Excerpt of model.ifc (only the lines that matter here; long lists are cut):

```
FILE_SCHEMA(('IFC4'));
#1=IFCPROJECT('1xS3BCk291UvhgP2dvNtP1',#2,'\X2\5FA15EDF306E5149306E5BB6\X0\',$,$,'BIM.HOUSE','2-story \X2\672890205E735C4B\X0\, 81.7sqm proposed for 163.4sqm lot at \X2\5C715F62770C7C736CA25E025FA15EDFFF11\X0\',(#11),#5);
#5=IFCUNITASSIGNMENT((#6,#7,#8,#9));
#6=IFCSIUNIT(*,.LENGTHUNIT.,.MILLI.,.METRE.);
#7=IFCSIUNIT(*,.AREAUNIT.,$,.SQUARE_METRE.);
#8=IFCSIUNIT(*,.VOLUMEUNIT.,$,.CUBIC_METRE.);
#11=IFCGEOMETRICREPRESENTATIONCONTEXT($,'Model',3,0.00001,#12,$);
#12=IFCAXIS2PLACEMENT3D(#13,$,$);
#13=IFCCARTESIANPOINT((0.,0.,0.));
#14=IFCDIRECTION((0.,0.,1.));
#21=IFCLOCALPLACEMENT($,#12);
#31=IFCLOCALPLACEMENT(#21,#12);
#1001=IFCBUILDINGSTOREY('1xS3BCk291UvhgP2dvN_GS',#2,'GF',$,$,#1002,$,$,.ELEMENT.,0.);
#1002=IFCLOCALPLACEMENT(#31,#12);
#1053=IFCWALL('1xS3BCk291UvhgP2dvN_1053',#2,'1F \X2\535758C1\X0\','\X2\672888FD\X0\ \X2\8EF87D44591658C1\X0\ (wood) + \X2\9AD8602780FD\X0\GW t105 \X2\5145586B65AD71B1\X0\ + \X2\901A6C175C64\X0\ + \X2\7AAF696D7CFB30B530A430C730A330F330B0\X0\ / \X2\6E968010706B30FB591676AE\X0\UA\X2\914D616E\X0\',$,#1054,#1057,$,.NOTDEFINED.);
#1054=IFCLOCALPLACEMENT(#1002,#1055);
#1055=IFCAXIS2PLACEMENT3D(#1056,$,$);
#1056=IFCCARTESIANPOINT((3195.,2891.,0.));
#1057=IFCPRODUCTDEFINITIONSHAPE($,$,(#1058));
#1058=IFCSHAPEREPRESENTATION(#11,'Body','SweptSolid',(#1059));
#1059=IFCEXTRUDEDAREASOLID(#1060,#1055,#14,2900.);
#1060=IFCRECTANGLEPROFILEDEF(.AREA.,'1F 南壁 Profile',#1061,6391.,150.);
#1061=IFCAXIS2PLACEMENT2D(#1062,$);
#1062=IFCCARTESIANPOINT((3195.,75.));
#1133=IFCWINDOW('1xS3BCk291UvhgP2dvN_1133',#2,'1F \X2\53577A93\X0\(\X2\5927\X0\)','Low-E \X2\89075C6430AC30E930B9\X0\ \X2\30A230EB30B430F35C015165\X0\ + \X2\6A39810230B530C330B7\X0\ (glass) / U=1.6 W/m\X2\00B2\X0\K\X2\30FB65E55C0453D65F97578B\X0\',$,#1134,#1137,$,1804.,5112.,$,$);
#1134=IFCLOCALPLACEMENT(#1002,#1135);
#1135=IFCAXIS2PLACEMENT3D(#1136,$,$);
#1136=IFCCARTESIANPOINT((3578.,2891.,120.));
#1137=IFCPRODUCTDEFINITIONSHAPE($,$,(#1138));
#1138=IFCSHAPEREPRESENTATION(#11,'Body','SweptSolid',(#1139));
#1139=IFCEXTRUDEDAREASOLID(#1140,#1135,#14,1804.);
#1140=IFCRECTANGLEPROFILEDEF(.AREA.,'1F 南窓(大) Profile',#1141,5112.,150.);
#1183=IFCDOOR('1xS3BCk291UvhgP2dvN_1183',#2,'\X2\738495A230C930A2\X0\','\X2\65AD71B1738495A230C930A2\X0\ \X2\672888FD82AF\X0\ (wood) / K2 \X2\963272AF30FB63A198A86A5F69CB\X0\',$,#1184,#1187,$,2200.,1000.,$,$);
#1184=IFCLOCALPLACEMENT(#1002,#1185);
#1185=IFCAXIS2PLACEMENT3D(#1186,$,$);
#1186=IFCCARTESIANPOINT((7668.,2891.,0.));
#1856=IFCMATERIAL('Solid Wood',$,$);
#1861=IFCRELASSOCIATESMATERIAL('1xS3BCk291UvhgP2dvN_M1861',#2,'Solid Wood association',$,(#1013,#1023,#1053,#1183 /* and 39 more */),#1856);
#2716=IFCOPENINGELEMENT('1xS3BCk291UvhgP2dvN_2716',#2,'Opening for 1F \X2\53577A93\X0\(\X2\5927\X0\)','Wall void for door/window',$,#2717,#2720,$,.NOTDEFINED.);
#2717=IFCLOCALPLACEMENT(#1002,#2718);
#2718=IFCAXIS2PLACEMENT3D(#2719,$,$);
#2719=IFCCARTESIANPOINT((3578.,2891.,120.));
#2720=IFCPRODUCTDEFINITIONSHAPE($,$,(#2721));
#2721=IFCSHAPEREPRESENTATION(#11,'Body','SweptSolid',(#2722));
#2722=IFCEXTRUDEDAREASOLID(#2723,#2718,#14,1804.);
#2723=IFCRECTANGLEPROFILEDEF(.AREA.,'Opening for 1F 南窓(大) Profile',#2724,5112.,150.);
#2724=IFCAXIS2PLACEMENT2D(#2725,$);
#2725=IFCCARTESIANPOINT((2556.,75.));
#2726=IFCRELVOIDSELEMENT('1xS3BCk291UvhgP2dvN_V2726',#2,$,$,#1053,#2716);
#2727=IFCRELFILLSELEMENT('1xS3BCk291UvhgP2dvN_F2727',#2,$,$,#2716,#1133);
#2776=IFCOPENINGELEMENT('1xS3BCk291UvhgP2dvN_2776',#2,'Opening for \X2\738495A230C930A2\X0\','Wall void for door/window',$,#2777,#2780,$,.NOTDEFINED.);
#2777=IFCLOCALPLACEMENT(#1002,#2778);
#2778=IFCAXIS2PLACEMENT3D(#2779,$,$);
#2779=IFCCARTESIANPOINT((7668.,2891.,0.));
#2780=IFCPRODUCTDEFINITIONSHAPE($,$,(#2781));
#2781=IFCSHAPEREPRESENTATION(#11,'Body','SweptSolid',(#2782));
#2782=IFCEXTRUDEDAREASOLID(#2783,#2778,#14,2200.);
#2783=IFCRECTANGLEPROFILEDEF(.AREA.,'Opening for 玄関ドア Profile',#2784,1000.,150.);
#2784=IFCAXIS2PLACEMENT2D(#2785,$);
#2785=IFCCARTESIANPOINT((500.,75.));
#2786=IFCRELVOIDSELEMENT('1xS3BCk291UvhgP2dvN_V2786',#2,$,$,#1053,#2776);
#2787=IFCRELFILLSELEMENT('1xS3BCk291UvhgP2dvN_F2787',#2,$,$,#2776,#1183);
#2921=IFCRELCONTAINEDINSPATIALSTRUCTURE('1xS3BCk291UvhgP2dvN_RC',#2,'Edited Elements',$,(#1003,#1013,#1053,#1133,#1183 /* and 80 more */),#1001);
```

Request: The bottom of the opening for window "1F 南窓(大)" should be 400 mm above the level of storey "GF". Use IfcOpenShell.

```python
import numpy as np
import ifcopenshell
import ifcopenshell.api.geometry
import ifcopenshell.geom
import ifcopenshell.util.element
import ifcopenshell.util.placement
import ifcopenshell.util.shape
import ifcopenshell.util.unit

model = ifcopenshell.open("model.ifc")
unit_scale = ifcopenshell.util.unit.calculate_unit_scale(model)

window = model.by_id(1133)
opening = window.FillsVoids[0].RelatingOpeningElement
storey = ifcopenshell.util.element.get_container(window, ifc_class="IfcBuildingStorey")
level = ifcopenshell.util.placement.get_local_placement(storey.ObjectPlacement)[2, 3]

# The opening's origin need not be at the sill, so measure its lowest point.
shape = ifcopenshell.geom.create_shape(ifcopenshell.geom.settings(), opening)
bottom = ifcopenshell.util.shape.get_shape_bottom_elevation(shape, shape.geometry) / unit_scale
dz = level + 0.4 / unit_scale - bottom

shift = np.array([0.0, 0.0, dz])
# The window is not placed relative to its opening, so move both.
for product in (opening, window):
    matrix = ifcopenshell.util.placement.get_local_placement(product.ObjectPlacement)
    matrix[:3, 3] += shift
    ifcopenshell.api.geometry.edit_object_placement(model, product=product, matrix=matrix, is_si=False)

print(f"moved by {dz * unit_scale:+.3f} m")

model.write("model-out.ifc")
```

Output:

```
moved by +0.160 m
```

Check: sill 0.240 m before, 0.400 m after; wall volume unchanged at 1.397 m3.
